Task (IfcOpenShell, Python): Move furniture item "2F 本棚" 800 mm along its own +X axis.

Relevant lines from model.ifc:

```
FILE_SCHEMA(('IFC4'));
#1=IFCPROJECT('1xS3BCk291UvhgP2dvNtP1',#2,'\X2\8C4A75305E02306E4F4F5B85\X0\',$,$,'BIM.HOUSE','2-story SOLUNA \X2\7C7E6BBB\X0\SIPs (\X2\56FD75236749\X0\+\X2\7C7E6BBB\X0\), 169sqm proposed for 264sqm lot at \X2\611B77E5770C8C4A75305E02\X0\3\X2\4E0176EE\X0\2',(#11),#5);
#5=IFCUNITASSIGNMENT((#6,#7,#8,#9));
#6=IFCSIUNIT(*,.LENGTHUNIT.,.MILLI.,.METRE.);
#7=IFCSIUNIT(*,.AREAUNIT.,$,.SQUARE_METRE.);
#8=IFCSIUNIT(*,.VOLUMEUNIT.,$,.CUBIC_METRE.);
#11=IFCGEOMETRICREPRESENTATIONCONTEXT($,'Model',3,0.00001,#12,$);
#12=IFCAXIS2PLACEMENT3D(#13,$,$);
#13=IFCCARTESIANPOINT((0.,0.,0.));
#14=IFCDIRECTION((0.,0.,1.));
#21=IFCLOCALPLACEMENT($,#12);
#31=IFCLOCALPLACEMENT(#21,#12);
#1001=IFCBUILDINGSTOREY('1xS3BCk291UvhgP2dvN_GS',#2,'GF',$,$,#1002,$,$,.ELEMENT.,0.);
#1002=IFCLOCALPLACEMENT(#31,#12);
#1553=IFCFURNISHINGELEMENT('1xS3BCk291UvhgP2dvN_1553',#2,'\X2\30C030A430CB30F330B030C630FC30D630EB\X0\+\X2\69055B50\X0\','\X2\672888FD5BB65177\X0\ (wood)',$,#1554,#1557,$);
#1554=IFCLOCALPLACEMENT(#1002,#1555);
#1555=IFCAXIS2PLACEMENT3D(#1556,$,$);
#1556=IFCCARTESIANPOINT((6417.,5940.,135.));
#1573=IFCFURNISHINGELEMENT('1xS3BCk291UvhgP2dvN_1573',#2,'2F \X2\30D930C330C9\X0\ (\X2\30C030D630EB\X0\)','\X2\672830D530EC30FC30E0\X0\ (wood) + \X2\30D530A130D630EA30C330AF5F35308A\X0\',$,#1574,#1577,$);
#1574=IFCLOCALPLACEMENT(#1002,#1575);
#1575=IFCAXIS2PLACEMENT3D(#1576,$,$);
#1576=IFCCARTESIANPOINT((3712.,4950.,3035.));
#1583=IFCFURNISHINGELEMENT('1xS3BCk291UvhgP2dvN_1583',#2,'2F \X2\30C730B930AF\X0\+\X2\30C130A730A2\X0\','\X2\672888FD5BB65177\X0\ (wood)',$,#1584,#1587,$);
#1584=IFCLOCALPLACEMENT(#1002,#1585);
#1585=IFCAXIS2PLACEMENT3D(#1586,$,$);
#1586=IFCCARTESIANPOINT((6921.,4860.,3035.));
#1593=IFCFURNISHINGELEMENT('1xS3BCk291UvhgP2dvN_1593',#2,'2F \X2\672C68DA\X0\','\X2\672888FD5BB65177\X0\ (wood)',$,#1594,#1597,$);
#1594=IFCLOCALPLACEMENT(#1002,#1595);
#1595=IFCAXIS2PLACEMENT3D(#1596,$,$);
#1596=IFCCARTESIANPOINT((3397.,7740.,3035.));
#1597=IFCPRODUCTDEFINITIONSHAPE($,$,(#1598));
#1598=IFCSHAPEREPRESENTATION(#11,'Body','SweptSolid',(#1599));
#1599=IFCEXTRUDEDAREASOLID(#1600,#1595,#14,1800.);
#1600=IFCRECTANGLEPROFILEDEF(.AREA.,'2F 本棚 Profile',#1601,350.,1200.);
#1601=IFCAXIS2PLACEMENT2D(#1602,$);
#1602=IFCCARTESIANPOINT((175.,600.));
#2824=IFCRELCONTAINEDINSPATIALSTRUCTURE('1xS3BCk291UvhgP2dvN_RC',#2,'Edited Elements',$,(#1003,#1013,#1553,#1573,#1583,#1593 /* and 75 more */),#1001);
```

```python
import ifcopenshell
import ifcopenshell.api.geometry
import ifcopenshell.util.placement
import ifcopenshell.util.unit

model = ifcopenshell.open("model.ifc")
unit_scale = ifcopenshell.util.unit.calculate_unit_scale(model)

item = model.by_id(1593)
matrix = ifcopenshell.util.placement.get_local_placement(item.ObjectPlacement)
matrix[:3, 3] += matrix[:3, 0] * 0.8 / unit_scale
ifcopenshell.api.geometry.edit_object_placement(model, product=item, matrix=matrix, is_si=False)

print(ifcopenshell.util.placement.get_local_placement(item.ObjectPlacement).round(3) + 0.0)

model.write("model_v2.ifc")
```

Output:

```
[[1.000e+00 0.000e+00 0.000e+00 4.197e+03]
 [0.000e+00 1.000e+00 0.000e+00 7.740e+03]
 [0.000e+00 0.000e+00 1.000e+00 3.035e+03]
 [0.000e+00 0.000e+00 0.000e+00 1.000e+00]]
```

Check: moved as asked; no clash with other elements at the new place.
